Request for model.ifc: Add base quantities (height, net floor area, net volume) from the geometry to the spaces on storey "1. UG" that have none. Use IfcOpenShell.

First a look at what the model holds.

```python
import ifcopenshell
import ifcopenshell.util.element
import ifcopenshell.util.unit

model = ifcopenshell.open("model.ifc")
print(model.schema)
for unit_type in ("LENGTHUNIT", "AREAUNIT", "VOLUMEUNIT"):
    print(unit_type, ifcopenshell.util.unit.calculate_unit_scale(model, unit_type))
storey = next(s for s in model.by_type("IfcBuildingStorey") if s.Name == "1. UG")
spaces = [e for e in ifcopenshell.util.element.get_decomposition(storey) if e.is_a("IfcSpace")]
for e in sorted(spaces, key=lambda e: e.id()):
    print(e.id(), e.is_a(), e.Name, list(ifcopenshell.util.element.get_psets(e, qtos_only=True)), sep=" | ")
```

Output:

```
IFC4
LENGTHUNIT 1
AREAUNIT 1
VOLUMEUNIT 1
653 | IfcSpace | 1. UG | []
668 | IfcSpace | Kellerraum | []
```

```python
import ifcopenshell
import ifcopenshell.api.pset
import ifcopenshell.geom
import ifcopenshell.util.element
import ifcopenshell.util.shape
import ifcopenshell.util.unit

model = ifcopenshell.open("model.ifc")
unit_scale = ifcopenshell.util.unit.calculate_unit_scale(model)
area_scale = ifcopenshell.util.unit.calculate_unit_scale(model, "AREAUNIT")
volume_scale = ifcopenshell.util.unit.calculate_unit_scale(model, "VOLUMEUNIT")
settings = ifcopenshell.geom.settings()

storey = next(s for s in model.by_type("IfcBuildingStorey") if s.Name == "1. UG")
spaces = [e for e in ifcopenshell.util.element.get_decomposition(storey) if e.is_a("IfcSpace")]

for e in sorted(spaces, key=lambda e: e.id()):
    if ifcopenshell.util.element.get_psets(e, qtos_only=True, should_inherit=False):
        continue
    # Geometry comes back in metres, in the element's own axes.
    shape = ifcopenshell.geom.create_shape(settings, e)
    values = {
        "Height": ifcopenshell.util.shape.get_z(shape.geometry) / unit_scale,
        "NetFloorArea": ifcopenshell.util.shape.get_footprint_area(shape.geometry) / area_scale,
        "NetVolume": ifcopenshell.util.shape.get_volume(shape.geometry) / volume_scale,
    }
    qto = ifcopenshell.api.pset.add_qto(model, product=e, name="Qto_SpaceBaseQuantities")
    ifcopenshell.api.pset.edit_qto(model, qto=qto, properties=values)
    print(e.id(), {k: round(v, 3) for k, v in values.items()})

model.write("model-out.ifc")
```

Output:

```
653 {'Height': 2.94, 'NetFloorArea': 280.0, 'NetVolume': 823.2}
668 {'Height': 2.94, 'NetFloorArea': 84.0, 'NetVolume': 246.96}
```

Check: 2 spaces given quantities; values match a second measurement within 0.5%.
